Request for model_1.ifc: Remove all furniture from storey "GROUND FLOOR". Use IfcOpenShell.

First a look at what the model holds.

```python
import ifcopenshell
import ifcopenshell.util.element

model = ifcopenshell.open("model_1.ifc")
print(model.schema)
storey = next(s for s in model.by_type("IfcBuildingStorey") if s.Name == "GROUND FLOOR")
furniture = [e for e in ifcopenshell.util.element.get_decomposition(storey) if e.is_a("IfcFurnishingElement")]
seen = {}
for e in furniture:
    element_type = ifcopenshell.util.element.get_type(e)
    name = element_type.Name if element_type not in (None, e) else None
    seen[name] = seen.get(name, 0) + 1
for name, count in sorted(seen.items(), key=str):
    print(count, "x", name)
```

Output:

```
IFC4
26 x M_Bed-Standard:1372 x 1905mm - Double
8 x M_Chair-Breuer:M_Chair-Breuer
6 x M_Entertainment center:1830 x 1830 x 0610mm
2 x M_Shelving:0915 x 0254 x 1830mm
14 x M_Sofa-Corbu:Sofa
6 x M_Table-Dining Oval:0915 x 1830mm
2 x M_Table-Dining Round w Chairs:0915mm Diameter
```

```python
import ifcopenshell
import ifcopenshell.api.root
import ifcopenshell.util.element

model = ifcopenshell.open("model_1.ifc")

storey = next(s for s in model.by_type("IfcBuildingStorey") if s.Name == "GROUND FLOOR")
furniture = [e for e in ifcopenshell.util.element.get_decomposition(storey) if e.is_a("IfcFurnishingElement")]

for e in furniture:
    ifcopenshell.api.root.remove_product(model, product=e)
print(len(furniture), "removed")

model.write("model_1_v2.ifc")
```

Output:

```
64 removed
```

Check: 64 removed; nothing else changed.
